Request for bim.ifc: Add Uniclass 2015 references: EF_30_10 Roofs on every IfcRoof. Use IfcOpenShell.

First a look at what the model holds.

```python
import ifcopenshell

model = ifcopenshell.open("bim.ifc")
print(model.schema)
print("classifications:", [c.Name for c in model.by_type("IfcClassification")])
for ifc_class in ("IfcDoor", "IfcRoof", "IfcStair", "IfcWall", "IfcWindow"):
    print(ifc_class, len(model.by_type(ifc_class)))
```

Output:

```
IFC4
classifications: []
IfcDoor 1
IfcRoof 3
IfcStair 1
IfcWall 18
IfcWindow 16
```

```python
import ifcopenshell
import ifcopenshell.api.classification

model = ifcopenshell.open("bim.ifc")

system = ifcopenshell.api.classification.add_classification(model, classification="Uniclass 2015")

codes = {
    "IfcRoof": ("EF_30_10", "Roofs"),
}
for ifc_class, (code, name) in codes.items():
    products = model.by_type(ifc_class)
    ifcopenshell.api.classification.add_reference(
        model, products=products, classification=system, identification=code, name=name
    )
    print(code, len(products))

model.write("bim-out.ifc")
```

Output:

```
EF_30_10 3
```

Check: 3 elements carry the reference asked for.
